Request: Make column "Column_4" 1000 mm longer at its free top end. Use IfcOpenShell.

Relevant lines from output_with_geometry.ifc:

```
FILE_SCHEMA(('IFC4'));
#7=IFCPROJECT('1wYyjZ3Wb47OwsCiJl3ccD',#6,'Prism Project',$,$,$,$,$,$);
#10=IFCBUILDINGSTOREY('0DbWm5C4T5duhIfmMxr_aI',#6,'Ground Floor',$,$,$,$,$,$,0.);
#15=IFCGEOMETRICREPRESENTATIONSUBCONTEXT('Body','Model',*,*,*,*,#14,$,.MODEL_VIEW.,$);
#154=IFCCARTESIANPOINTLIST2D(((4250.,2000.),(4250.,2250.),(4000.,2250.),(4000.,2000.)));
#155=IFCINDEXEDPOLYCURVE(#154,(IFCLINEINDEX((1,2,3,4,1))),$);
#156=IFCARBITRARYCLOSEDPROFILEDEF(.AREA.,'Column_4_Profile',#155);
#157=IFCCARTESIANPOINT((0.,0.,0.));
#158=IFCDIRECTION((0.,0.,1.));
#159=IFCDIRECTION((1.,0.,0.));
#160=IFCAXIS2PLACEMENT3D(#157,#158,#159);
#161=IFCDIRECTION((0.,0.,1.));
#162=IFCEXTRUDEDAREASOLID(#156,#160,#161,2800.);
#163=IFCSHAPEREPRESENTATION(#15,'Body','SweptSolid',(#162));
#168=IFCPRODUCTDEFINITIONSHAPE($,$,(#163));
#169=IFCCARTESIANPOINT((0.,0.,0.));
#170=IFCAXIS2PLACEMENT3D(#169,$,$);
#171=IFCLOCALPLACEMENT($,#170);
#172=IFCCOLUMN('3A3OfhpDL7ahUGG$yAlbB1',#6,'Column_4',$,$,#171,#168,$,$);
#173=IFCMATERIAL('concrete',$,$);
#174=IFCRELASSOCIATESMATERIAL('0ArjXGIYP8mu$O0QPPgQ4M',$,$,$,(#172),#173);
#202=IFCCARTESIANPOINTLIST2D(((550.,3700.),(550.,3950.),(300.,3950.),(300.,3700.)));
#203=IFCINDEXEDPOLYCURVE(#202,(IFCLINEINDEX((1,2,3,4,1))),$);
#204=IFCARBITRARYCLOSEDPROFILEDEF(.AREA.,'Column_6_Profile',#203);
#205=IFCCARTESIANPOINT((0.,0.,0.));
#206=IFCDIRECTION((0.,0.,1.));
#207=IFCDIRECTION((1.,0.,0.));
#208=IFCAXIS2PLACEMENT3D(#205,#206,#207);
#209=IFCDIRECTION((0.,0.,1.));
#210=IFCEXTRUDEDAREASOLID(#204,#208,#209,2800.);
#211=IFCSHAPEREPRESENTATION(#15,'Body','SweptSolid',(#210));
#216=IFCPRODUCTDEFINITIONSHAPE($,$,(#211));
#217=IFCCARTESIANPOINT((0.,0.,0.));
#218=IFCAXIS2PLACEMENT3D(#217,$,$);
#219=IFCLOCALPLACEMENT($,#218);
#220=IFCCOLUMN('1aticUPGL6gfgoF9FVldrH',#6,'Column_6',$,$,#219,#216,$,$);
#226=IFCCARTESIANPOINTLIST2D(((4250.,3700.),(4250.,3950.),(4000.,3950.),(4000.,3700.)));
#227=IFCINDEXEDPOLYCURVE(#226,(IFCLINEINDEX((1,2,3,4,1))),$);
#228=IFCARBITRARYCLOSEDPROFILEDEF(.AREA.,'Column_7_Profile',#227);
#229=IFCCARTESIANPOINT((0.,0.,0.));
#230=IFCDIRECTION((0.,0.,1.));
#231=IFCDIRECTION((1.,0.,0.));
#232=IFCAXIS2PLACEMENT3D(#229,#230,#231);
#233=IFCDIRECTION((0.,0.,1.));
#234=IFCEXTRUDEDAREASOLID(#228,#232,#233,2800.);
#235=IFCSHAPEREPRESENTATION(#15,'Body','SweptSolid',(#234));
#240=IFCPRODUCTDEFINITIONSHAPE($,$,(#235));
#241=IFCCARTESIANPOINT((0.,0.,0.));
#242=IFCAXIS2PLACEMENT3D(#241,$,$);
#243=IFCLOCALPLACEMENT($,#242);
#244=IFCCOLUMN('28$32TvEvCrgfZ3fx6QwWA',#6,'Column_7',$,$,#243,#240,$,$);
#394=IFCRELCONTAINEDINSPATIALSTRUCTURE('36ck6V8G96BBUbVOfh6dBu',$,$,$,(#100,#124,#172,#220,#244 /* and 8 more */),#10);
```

```python
import ifcopenshell
import ifcopenshell.util.representation
import ifcopenshell.util.unit

model = ifcopenshell.open("output_with_geometry.ifc")
unit_scale = ifcopenshell.util.unit.calculate_unit_scale(model)

member = model.by_guid("3A3OfhpDL7ahUGG$yAlbB1")
change = 1 / unit_scale

# The extrusion runs towards the end named, so only its depth changes.
body = ifcopenshell.util.representation.get_representation(member, "Model", "Body")
solid = body.Items[0]
old_length = solid.Depth
solid.Depth += change

print(f"length {old_length:g} -> {solid.Depth:g}")

model.write("output_with_geometry_updated.ifc")
```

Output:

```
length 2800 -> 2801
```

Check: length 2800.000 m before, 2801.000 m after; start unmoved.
